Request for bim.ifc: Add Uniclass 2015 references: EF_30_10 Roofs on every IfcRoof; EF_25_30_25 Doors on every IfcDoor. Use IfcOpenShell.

First a look at what the model holds.

```python
import ifcopenshell

model = ifcopenshell.open("bim.ifc")
print(model.schema)
print("classifications:", [c.Name for c in model.by_type("IfcClassification")])
for ifc_class in ("IfcDoor", "IfcRoof", "IfcStair", "IfcWall", "IfcWindow"):
    print(ifc_class, len(model.by_type(ifc_class)))
```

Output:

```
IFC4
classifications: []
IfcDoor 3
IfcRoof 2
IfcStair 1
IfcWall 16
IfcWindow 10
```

```python
import ifcopenshell
import ifcopenshell.api.classification

model = ifcopenshell.open("bim.ifc")

system = ifcopenshell.api.classification.add_classification(model, classification="Uniclass 2015")

codes = {
    "IfcRoof": ("EF_30_10", "Roofs"),
    "IfcDoor": ("EF_25_30_25", "Doors"),
}
for ifc_class, (code, name) in codes.items():
    products = model.by_type(ifc_class)
    ifcopenshell.api.classification.add_reference(
        model, products=products, classification=system, identification=code, name=name
    )
    print(code, len(products))

model.write("bim-out.ifc")
```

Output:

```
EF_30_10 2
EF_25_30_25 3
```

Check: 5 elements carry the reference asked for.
